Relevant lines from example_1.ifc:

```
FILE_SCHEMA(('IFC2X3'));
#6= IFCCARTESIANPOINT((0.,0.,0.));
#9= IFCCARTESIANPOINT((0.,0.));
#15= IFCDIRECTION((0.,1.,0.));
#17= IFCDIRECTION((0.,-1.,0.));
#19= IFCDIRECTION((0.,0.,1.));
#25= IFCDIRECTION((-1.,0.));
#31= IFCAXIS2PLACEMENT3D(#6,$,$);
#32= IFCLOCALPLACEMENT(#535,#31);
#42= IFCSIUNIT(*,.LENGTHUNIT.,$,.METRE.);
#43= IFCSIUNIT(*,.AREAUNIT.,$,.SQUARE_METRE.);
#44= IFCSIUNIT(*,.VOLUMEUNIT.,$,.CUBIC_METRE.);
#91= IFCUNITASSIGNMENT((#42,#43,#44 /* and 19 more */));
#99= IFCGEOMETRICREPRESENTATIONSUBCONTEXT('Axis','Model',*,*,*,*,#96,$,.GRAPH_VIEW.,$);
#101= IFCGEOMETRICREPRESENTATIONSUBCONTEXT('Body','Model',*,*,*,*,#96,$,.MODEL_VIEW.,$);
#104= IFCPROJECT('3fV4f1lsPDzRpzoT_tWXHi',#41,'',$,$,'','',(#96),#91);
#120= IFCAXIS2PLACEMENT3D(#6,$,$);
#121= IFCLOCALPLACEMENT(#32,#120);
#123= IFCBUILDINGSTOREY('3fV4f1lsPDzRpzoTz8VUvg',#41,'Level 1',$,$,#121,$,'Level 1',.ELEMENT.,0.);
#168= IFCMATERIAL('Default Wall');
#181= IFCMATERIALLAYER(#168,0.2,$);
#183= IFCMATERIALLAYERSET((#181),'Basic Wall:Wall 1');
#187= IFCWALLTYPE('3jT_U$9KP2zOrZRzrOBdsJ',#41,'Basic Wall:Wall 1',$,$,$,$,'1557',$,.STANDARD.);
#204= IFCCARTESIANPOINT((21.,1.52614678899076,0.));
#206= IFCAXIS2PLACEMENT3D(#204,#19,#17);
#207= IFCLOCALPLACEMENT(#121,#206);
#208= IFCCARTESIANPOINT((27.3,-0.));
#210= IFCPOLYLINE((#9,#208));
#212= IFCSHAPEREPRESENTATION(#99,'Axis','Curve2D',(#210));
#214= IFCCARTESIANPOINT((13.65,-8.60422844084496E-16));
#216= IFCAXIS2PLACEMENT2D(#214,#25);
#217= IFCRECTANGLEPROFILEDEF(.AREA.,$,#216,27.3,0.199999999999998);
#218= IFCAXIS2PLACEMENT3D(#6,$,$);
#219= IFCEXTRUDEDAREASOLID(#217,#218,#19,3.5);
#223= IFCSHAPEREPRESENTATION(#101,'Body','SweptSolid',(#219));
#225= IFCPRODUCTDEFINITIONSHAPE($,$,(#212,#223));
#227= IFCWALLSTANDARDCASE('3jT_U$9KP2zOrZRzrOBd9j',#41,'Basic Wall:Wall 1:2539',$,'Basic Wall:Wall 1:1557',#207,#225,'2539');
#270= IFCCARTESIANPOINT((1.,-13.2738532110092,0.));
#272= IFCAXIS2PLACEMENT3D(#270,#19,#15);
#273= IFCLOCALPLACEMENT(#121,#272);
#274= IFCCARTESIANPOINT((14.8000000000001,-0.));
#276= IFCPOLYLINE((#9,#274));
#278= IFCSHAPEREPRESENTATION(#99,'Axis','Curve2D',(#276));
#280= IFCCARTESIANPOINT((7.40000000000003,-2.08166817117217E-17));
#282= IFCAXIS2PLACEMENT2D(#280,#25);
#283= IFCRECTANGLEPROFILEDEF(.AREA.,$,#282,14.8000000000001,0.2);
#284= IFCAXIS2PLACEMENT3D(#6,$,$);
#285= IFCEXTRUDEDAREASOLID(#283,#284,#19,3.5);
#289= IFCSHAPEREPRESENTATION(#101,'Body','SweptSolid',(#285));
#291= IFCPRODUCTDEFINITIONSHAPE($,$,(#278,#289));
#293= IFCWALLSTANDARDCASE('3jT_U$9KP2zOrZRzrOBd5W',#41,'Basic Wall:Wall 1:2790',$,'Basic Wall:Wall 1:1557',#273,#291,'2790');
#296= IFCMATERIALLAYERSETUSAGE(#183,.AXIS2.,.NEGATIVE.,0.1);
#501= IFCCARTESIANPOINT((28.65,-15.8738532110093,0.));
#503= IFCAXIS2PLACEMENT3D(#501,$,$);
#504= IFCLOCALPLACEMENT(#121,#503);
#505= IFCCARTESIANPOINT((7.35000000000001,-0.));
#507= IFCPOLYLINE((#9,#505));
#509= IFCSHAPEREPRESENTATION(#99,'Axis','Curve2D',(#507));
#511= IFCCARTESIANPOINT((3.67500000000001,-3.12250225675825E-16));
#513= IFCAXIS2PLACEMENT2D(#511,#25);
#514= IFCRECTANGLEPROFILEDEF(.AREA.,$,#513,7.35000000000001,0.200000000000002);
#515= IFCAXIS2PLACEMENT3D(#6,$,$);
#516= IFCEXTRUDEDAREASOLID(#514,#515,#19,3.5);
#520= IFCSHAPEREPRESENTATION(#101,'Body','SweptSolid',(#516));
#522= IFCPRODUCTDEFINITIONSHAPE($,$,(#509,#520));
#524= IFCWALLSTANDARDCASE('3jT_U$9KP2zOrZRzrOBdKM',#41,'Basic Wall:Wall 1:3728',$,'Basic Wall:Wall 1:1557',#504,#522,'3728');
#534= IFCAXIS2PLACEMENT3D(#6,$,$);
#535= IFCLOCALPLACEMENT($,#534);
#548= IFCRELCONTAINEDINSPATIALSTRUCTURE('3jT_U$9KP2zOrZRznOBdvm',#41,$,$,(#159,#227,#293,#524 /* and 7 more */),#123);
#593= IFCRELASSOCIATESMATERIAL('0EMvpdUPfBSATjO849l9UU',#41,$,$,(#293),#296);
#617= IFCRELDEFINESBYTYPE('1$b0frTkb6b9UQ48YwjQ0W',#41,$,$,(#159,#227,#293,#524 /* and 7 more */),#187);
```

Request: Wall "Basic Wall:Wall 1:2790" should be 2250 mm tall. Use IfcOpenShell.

```python
import ifcopenshell
import ifcopenshell.geom
import ifcopenshell.util.representation
import ifcopenshell.util.shape
import ifcopenshell.util.unit

model = ifcopenshell.open("example_1.ifc")
unit_scale = ifcopenshell.util.unit.calculate_unit_scale(model)
settings = ifcopenshell.geom.settings()


def volume(element):
    """Net volume in cubic metres, openings subtracted."""
    shape = ifcopenshell.geom.create_shape(settings, element)
    return ifcopenshell.util.shape.get_volume(shape.geometry)


wall = model.by_guid("3jT_U$9KP2zOrZRzrOBd5W")
before = volume(wall)

body = ifcopenshell.util.representation.get_representation(wall, "Model", "Body")
solid = body.Items[0]
old_height = solid.Depth
solid.Depth = 2.25 / unit_scale
after = volume(wall)

print(f"height {old_height:g} -> {solid.Depth:g}, volume {before:.3f} -> {after:.3f} m3")

model.write("example_1_rev.ifc")
```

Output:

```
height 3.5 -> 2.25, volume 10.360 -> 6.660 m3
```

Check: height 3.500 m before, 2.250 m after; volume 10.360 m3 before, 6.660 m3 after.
